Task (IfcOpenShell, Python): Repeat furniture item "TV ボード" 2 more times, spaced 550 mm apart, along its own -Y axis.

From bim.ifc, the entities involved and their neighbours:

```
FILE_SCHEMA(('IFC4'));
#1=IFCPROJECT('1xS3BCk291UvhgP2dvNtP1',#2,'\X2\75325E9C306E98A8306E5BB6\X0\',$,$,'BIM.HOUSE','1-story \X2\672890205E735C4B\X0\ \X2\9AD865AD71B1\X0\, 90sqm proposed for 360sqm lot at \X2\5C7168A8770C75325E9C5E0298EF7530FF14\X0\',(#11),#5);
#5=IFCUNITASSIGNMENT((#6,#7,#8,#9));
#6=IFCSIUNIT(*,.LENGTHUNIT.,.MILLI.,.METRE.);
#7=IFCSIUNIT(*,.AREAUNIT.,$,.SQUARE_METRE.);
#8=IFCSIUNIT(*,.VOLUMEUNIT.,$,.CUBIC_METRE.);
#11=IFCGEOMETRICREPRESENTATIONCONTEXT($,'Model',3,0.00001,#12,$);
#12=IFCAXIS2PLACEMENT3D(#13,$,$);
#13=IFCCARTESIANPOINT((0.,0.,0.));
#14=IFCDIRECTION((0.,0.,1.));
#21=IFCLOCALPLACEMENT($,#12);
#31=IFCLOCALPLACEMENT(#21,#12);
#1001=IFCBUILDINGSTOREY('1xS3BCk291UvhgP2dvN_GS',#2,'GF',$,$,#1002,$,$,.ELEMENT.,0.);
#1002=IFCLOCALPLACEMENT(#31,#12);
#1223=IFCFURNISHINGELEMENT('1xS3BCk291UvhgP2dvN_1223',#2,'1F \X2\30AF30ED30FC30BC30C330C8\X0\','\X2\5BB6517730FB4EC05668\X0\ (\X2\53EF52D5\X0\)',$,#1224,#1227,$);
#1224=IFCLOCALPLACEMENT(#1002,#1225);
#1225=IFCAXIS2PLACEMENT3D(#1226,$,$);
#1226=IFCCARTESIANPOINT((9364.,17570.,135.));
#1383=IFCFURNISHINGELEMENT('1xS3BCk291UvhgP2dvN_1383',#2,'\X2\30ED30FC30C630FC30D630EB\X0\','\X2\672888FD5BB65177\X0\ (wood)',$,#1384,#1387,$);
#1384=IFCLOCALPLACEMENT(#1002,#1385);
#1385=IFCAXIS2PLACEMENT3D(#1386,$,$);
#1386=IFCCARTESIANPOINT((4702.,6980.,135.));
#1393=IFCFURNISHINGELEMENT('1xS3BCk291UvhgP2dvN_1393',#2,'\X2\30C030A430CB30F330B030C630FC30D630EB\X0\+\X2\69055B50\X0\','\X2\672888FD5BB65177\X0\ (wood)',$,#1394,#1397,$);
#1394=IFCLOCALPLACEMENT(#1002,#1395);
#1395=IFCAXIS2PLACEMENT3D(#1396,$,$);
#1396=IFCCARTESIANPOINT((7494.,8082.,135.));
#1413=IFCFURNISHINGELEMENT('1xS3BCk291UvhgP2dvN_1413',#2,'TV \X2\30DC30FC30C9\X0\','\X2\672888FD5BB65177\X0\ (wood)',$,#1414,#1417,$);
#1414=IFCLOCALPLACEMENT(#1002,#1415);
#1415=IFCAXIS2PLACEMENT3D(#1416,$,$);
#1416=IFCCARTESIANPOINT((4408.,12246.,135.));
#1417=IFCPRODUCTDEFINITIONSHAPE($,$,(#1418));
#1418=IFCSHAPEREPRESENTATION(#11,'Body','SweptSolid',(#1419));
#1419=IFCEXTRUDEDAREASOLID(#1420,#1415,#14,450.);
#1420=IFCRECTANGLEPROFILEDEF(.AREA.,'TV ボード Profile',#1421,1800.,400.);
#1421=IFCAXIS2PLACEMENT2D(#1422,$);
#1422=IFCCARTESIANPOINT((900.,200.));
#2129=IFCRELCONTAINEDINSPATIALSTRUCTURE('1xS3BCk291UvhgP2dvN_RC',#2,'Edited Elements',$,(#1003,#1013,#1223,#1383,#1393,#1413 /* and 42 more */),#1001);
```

```python
import ifcopenshell
import ifcopenshell.api.geometry
import ifcopenshell.api.root
import ifcopenshell.util.element
import ifcopenshell.util.placement
import ifcopenshell.util.unit

model = ifcopenshell.open("bim.ifc")
unit_scale = ifcopenshell.util.unit.calculate_unit_scale(model)


def reuse_history(source, copy):
    """copy_class also copies each property set's owner history, people and application; keep the originals."""
    for rel in copy.IsDefinedBy:
        if rel.is_a("IfcRelDefinesByProperties") and (history := rel.RelatingPropertyDefinition.OwnerHistory):
            rel.RelatingPropertyDefinition.OwnerHistory = source.OwnerHistory
            ifcopenshell.util.element.remove_deep2(model, history)


source = model.by_id(1413)
base = ifcopenshell.util.placement.get_local_placement(source.ObjectPlacement)
step = -base[:3, 1] * 0.55 / unit_scale

for i in range(1, 3):
    copy = ifcopenshell.api.root.copy_class(model, product=source)
    copy.Representation = ifcopenshell.util.element.copy_deep(
        model, source.Representation, exclude=["IfcGeometricRepresentationContext", "IfcRepresentationMap"]
    )
    reuse_history(source, copy)
    matrix = base.copy()
    matrix[:3, 3] += i * step
    print("added at", matrix[:3, 3].round(3) + 0.0)
    ifcopenshell.api.geometry.edit_object_placement(model, product=copy, matrix=matrix, is_si=False)

model.write("bim_updated.ifc")
```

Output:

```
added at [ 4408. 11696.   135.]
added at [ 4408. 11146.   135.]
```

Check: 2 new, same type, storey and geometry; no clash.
